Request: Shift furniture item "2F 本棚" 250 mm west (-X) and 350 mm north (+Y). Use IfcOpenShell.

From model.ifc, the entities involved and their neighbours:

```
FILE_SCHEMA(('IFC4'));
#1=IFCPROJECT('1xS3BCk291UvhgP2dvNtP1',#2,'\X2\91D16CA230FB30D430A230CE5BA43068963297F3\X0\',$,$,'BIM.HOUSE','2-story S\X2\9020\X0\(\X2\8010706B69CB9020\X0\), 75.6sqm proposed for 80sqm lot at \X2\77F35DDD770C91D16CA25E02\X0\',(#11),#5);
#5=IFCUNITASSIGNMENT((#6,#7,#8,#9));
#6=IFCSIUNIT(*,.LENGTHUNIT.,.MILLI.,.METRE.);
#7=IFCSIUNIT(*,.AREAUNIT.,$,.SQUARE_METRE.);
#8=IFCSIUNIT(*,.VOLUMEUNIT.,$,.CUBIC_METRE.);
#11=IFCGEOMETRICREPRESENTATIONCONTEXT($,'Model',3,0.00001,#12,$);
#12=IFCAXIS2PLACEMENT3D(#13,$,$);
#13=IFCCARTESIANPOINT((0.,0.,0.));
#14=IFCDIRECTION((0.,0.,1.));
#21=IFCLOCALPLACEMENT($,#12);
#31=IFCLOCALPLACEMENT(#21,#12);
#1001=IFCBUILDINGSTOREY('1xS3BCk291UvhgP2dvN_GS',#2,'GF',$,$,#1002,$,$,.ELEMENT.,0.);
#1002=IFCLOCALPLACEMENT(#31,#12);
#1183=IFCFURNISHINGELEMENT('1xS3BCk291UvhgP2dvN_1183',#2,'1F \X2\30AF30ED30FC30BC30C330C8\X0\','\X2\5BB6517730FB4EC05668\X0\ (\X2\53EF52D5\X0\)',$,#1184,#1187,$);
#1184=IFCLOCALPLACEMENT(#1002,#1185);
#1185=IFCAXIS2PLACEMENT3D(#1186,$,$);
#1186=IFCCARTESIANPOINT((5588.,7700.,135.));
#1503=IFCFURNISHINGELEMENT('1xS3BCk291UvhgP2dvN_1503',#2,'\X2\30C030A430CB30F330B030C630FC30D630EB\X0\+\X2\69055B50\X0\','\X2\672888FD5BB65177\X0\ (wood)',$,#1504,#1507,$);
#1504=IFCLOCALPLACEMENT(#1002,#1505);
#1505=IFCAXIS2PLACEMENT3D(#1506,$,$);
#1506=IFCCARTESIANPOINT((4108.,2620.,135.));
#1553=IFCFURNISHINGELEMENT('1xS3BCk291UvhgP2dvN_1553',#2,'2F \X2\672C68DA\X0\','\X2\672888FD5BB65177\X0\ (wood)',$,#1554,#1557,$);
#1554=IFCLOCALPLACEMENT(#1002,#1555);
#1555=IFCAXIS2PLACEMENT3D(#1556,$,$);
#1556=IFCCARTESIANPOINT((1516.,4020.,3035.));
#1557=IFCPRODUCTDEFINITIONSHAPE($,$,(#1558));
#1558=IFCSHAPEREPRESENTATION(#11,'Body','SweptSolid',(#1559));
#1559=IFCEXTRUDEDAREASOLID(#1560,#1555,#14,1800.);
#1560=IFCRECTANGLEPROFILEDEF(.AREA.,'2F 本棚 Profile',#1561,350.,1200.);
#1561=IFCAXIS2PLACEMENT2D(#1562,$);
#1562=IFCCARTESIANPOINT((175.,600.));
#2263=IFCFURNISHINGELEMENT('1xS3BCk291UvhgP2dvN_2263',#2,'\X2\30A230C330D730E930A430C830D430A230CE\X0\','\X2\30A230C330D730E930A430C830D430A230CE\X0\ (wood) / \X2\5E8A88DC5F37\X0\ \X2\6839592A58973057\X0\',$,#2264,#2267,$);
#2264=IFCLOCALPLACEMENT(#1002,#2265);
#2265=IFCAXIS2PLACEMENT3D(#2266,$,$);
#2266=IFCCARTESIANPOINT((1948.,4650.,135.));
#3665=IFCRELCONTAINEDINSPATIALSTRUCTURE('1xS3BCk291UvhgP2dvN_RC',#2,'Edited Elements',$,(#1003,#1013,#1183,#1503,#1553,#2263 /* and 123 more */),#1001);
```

```python
import ifcopenshell
import ifcopenshell.api.geometry
import ifcopenshell.util.placement
import ifcopenshell.util.unit

model = ifcopenshell.open("model.ifc")
unit_scale = ifcopenshell.util.unit.calculate_unit_scale(model)

item = model.by_id(1553)
matrix = ifcopenshell.util.placement.get_local_placement(item.ObjectPlacement)
matrix[0, 3] -= 0.25 / unit_scale
matrix[1, 3] += 0.35 / unit_scale
ifcopenshell.api.geometry.edit_object_placement(model, product=item, matrix=matrix, is_si=False)

print(ifcopenshell.util.placement.get_local_placement(item.ObjectPlacement).round(3) + 0.0)

model.write("model-out.ifc")
```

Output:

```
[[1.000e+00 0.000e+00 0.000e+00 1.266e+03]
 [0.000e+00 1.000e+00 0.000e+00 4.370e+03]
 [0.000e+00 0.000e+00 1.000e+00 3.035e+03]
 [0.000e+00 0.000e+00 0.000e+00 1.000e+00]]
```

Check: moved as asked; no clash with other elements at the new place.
